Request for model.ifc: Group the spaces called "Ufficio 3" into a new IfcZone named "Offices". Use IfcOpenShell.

First a look at what the model holds.

```python
import ifcopenshell

model = ifcopenshell.open("model.ifc")
print(model.schema)
seen = {}
for space in model.by_type("IfcSpace"):
    seen[space.LongName] = seen.get(space.LongName, 0) + 1
for name, count in sorted(seen.items(), key=str):
    print(count, "x", name)
print("zones:", [z.Name for z in model.by_type("IfcZone")][:20])
```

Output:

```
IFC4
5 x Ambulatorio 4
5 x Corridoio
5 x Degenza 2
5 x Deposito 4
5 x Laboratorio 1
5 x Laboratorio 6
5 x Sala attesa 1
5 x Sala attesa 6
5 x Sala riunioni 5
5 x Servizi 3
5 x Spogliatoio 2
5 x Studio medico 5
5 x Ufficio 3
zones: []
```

```python
import ifcopenshell
import ifcopenshell.api.group
import ifcopenshell.api.root

model = ifcopenshell.open("model.ifc")

names = {"Ufficio 3"}
spaces = [s for s in model.by_type("IfcSpace") if s.LongName in names]

zone = ifcopenshell.api.root.create_entity(model, ifc_class="IfcZone", name="Offices")
ifcopenshell.api.group.assign_group(model, products=spaces, group=zone)
print(len(spaces), "spaces in", zone.Name)

model.write("model_updated.ifc")
```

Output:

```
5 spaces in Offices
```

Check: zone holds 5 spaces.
